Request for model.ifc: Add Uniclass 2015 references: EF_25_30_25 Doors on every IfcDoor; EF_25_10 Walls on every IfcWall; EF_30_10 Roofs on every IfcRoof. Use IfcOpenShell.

First a look at what the model holds.

```python
import ifcopenshell

model = ifcopenshell.open("model.ifc")
print(model.schema)
print("classifications:", [c.Name for c in model.by_type("IfcClassification")])
for ifc_class in ("IfcDoor", "IfcRoof", "IfcStair", "IfcWall", "IfcWindow"):
    print(ifc_class, len(model.by_type(ifc_class)))
```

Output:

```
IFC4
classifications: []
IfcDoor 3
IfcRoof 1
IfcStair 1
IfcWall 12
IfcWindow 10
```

```python
import ifcopenshell
import ifcopenshell.api.classification

model = ifcopenshell.open("model.ifc")

system = ifcopenshell.api.classification.add_classification(model, classification="Uniclass 2015")

codes = {
    "IfcDoor": ("EF_25_30_25", "Doors"),
    "IfcWall": ("EF_25_10", "Walls"),
    "IfcRoof": ("EF_30_10", "Roofs"),
}
for ifc_class, (code, name) in codes.items():
    products = model.by_type(ifc_class)
    ifcopenshell.api.classification.add_reference(
        model, products=products, classification=system, identification=code, name=name
    )
    print(code, len(products))

model.write("model_v2.ifc")
```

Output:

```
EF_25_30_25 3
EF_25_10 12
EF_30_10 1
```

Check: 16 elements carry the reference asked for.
